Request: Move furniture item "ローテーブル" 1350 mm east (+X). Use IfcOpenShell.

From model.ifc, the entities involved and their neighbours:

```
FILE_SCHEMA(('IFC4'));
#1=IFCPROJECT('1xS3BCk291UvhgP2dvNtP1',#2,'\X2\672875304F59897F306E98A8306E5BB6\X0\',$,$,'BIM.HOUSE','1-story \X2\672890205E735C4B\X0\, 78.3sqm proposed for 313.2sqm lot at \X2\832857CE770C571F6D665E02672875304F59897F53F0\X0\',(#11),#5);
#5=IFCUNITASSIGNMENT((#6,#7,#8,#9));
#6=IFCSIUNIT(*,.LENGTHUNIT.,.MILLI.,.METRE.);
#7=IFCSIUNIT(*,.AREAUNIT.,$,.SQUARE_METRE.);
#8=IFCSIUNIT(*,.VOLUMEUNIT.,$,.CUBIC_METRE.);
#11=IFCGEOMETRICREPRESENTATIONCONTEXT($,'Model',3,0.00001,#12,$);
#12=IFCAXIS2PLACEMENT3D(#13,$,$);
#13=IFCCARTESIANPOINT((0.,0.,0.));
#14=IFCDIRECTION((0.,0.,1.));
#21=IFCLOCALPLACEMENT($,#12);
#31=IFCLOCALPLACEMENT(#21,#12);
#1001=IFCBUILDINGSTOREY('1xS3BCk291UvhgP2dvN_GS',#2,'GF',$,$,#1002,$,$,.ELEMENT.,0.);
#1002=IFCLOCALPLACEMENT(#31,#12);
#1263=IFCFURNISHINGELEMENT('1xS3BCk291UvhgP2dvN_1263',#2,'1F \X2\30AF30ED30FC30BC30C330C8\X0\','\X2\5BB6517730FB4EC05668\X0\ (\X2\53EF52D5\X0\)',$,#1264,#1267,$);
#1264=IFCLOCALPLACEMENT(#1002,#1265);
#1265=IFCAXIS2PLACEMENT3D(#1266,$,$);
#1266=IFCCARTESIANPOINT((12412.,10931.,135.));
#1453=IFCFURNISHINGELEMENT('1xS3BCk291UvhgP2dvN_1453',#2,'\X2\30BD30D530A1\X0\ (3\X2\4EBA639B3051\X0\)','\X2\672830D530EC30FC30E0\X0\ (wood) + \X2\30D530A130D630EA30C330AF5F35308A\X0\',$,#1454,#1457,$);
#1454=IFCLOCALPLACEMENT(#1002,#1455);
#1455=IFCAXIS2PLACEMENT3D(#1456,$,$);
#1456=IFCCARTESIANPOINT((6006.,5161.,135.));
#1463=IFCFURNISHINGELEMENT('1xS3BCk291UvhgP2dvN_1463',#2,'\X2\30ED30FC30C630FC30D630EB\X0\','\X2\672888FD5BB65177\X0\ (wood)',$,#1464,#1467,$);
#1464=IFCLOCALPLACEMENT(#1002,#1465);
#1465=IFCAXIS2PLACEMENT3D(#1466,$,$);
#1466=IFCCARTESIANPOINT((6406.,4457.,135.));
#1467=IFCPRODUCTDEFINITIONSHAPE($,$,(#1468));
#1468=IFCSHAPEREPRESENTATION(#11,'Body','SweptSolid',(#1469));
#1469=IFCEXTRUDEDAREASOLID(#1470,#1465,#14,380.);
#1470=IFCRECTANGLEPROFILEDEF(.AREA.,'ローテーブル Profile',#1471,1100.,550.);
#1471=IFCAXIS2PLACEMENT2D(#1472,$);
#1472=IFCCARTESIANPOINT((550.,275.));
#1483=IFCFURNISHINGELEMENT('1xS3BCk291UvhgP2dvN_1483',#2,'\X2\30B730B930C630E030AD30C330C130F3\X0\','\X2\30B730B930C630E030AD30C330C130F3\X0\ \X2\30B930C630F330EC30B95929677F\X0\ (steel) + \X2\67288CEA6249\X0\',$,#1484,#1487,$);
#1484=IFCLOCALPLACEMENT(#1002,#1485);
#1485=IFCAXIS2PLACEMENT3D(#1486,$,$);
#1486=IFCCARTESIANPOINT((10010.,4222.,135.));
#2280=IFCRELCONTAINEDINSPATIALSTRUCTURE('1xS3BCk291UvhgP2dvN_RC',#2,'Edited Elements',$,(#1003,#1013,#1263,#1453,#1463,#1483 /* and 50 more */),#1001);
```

```python
import ifcopenshell
import ifcopenshell.api.geometry
import ifcopenshell.util.placement
import ifcopenshell.util.unit

model = ifcopenshell.open("model.ifc")
unit_scale = ifcopenshell.util.unit.calculate_unit_scale(model)

item = model.by_guid("1xS3BCk291UvhgP2dvN_1463")
matrix = ifcopenshell.util.placement.get_local_placement(item.ObjectPlacement)
matrix[0, 3] += 1.35 / unit_scale
ifcopenshell.api.geometry.edit_object_placement(model, product=item, matrix=matrix, is_si=False)

print(ifcopenshell.util.placement.get_local_placement(item.ObjectPlacement).round(3) + 0.0)

model.write("model_updated.ifc")
```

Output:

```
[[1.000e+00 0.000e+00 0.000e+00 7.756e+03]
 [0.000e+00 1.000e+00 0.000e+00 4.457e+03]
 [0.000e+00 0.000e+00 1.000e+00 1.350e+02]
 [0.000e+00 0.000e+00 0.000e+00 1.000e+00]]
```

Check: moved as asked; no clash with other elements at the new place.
